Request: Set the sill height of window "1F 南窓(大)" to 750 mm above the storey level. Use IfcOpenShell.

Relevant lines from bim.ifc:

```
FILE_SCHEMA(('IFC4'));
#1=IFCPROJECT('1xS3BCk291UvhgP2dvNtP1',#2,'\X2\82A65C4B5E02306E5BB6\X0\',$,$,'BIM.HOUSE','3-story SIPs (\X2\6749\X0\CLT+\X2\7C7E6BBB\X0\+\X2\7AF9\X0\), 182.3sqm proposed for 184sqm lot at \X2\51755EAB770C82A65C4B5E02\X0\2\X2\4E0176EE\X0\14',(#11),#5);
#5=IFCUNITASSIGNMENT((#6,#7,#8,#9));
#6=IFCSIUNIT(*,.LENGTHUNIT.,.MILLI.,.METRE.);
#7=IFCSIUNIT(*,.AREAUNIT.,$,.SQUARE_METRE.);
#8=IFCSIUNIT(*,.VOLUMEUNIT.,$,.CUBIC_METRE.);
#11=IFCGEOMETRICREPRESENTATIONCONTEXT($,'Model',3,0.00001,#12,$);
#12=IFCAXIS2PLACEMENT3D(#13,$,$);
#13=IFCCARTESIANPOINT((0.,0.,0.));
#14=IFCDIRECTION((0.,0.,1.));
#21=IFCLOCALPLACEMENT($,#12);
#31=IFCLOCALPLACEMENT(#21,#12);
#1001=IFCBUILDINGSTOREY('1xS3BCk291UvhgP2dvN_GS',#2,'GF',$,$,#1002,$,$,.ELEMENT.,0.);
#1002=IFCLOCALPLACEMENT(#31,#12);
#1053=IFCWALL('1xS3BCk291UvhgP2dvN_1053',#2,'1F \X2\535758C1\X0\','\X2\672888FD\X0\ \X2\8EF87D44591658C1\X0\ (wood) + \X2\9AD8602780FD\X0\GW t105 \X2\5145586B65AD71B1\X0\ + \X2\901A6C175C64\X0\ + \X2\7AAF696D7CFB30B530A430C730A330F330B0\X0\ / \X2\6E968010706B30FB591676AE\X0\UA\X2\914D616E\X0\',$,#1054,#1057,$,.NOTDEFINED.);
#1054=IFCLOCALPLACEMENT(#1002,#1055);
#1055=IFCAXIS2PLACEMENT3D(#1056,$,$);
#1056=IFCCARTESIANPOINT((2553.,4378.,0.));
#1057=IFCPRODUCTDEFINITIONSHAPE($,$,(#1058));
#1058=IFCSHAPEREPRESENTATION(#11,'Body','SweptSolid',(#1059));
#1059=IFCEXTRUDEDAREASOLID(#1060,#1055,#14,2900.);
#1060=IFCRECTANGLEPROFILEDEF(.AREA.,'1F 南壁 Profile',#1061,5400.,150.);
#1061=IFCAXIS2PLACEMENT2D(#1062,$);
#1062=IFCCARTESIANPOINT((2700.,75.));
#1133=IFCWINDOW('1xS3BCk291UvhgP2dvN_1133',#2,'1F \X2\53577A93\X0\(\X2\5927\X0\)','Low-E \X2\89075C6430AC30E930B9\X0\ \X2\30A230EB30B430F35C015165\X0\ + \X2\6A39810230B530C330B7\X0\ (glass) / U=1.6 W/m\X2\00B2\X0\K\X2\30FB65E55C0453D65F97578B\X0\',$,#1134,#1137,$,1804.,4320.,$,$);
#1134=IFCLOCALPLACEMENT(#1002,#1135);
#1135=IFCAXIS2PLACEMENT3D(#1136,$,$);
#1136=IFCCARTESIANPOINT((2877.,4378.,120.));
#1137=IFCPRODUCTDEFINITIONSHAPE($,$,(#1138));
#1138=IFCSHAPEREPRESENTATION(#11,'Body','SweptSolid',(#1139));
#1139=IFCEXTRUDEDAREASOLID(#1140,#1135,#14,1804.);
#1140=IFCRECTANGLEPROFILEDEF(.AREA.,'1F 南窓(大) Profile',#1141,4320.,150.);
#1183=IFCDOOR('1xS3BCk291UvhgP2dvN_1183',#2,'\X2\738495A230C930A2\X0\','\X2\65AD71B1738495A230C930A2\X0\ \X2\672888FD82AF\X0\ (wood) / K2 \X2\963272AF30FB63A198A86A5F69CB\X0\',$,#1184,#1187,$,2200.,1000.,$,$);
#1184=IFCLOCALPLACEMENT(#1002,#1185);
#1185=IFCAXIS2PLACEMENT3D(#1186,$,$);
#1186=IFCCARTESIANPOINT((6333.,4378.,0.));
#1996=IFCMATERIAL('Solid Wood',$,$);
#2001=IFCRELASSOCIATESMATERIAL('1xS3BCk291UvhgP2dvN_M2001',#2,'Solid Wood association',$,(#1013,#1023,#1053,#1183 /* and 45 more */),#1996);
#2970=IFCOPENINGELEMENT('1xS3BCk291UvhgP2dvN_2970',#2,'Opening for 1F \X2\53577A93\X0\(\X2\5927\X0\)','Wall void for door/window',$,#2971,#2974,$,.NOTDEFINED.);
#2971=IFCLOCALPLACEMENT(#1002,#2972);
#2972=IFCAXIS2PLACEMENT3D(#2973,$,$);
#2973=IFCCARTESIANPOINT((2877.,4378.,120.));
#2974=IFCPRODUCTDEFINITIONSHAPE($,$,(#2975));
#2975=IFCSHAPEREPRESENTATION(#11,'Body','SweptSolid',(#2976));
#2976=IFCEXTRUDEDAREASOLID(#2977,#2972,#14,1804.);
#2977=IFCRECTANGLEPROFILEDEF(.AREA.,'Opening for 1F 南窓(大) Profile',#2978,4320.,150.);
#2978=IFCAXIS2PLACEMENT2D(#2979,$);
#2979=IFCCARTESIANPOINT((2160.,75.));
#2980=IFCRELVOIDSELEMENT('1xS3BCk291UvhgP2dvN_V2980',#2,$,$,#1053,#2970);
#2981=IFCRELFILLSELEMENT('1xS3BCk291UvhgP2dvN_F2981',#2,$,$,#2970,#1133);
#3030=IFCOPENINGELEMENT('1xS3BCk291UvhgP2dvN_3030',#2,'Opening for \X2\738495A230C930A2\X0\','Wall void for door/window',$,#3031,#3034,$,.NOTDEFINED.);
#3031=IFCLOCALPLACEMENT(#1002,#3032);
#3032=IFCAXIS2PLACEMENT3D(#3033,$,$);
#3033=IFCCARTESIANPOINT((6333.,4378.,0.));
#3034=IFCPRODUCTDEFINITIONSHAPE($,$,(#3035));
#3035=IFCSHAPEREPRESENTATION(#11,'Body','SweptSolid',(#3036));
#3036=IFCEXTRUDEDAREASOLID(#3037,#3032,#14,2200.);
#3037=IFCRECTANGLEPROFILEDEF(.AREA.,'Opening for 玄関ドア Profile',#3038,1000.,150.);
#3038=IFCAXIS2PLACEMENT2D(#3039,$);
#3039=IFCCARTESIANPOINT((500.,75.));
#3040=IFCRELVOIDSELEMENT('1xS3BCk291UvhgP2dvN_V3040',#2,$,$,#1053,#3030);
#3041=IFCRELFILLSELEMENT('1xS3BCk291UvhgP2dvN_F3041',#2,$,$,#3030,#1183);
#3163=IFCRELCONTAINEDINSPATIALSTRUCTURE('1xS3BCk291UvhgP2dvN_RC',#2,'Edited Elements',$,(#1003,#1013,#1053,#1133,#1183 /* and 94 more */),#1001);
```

```python
import numpy as np
import ifcopenshell
import ifcopenshell.api.geometry
import ifcopenshell.geom
import ifcopenshell.util.element
import ifcopenshell.util.placement
import ifcopenshell.util.shape
import ifcopenshell.util.unit

model = ifcopenshell.open("bim.ifc")
unit_scale = ifcopenshell.util.unit.calculate_unit_scale(model)

window = model.by_id(1133)
opening = window.FillsVoids[0].RelatingOpeningElement
storey = ifcopenshell.util.element.get_container(window, ifc_class="IfcBuildingStorey")
level = ifcopenshell.util.placement.get_local_placement(storey.ObjectPlacement)[2, 3]

# The opening's origin need not be at the sill, so measure its lowest point.
shape = ifcopenshell.geom.create_shape(ifcopenshell.geom.settings(), opening)
bottom = ifcopenshell.util.shape.get_shape_bottom_elevation(shape, shape.geometry) / unit_scale
dz = level + 0.75 / unit_scale - bottom

shift = np.array([0.0, 0.0, dz])
# The window is not placed relative to its opening, so move both.
for product in (opening, window):
    matrix = ifcopenshell.util.placement.get_local_placement(product.ObjectPlacement)
    matrix[:3, 3] += shift
    ifcopenshell.api.geometry.edit_object_placement(model, product=product, matrix=matrix, is_si=False)

print(f"moved by {dz * unit_scale:+.3f} m")

model.write("bim_edited.ifc")
```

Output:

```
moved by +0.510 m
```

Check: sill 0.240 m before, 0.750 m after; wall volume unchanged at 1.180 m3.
